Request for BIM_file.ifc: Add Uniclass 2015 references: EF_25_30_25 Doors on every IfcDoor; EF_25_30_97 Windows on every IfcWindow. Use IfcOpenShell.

First a look at what the model holds.

```python
import ifcopenshell

model = ifcopenshell.open("BIM_file.ifc")
print(model.schema)
print("classifications:", [c.Name for c in model.by_type("IfcClassification")])
for ifc_class in ("IfcDoor", "IfcRoof", "IfcStair", "IfcWall", "IfcWindow"):
    print(ifc_class, len(model.by_type(ifc_class)))
```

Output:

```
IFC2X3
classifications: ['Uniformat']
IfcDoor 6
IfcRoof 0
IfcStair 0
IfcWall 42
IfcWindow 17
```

```python
import ifcopenshell
import ifcopenshell.api.classification

model = ifcopenshell.open("BIM_file.ifc")

# IFC2X3 requires Source and Edition and has no link from the project to the system.
system = model.create_entity("IfcClassification", Source="NBS", Edition="2015", Name="Uniclass 2015")

codes = {
    "IfcDoor": ("EF_25_30_25", "Doors"),
    "IfcWindow": ("EF_25_30_97", "Windows"),
}
for ifc_class, (code, name) in codes.items():
    products = model.by_type(ifc_class)
    ifcopenshell.api.classification.add_reference(
        model, products=products, classification=system, identification=code, name=name
    )
    print(code, len(products))

model.write("BIM_file-out.ifc")
```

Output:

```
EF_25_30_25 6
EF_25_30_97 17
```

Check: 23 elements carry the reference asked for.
